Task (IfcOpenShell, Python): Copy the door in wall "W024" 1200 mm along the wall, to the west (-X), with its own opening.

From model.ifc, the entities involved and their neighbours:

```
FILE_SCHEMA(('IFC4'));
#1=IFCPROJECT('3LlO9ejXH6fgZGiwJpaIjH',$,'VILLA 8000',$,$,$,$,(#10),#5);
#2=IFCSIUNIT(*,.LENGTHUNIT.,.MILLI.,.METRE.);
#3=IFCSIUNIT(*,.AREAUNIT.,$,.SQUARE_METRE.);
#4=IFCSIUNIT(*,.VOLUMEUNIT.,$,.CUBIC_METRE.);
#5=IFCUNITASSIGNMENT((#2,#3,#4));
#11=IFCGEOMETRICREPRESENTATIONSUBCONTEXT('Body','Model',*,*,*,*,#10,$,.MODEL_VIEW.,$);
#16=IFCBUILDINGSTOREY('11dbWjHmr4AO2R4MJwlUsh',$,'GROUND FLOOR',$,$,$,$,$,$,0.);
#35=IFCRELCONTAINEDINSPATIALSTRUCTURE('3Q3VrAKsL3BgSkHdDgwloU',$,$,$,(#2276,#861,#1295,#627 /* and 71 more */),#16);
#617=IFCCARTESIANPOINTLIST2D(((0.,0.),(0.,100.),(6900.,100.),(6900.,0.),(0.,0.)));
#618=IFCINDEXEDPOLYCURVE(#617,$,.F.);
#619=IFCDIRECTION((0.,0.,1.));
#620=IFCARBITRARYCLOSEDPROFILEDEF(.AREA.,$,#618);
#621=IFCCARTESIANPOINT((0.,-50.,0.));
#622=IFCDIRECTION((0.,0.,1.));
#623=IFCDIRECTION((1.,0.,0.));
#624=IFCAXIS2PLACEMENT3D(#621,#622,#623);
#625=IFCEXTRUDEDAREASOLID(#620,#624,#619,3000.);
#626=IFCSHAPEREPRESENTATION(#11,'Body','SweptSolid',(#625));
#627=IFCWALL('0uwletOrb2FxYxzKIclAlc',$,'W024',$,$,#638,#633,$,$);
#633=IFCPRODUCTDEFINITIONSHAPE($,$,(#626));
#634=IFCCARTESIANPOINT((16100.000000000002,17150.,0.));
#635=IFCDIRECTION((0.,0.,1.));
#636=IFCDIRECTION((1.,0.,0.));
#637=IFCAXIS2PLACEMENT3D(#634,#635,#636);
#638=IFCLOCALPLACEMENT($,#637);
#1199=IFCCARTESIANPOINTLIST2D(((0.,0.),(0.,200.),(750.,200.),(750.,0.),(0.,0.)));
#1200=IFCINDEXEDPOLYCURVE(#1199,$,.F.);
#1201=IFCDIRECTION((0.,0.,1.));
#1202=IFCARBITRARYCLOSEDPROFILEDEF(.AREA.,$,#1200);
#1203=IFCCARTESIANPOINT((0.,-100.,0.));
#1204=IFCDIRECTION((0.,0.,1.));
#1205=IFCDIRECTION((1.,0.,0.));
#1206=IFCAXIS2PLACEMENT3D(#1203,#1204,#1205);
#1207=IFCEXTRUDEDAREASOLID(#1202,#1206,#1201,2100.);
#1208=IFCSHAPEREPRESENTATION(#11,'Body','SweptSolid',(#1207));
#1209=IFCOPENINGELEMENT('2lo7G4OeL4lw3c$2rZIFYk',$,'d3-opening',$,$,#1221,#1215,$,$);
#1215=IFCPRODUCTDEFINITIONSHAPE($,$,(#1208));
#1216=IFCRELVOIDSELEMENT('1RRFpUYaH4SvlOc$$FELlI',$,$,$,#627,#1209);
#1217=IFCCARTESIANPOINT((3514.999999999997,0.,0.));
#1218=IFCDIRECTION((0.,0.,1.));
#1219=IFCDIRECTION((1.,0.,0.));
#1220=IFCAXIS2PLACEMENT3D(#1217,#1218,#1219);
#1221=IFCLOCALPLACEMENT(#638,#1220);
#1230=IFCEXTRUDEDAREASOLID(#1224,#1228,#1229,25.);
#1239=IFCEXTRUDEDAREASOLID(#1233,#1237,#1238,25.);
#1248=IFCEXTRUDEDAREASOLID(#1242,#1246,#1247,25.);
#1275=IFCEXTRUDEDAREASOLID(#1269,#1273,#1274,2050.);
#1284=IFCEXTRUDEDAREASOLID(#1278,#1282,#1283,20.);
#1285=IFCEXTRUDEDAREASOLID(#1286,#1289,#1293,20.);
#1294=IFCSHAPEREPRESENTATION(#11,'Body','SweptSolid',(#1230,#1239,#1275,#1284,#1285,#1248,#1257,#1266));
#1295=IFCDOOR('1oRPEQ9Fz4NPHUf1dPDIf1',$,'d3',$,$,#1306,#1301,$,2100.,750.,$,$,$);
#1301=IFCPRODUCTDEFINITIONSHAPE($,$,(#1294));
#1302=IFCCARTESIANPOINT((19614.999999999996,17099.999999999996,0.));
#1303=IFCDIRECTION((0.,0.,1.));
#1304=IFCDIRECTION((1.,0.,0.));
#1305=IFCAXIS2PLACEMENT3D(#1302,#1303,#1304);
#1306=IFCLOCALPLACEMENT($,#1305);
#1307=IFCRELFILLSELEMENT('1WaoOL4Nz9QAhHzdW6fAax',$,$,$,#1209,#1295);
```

```python
import ifcopenshell
import ifcopenshell.api.feature
import ifcopenshell.api.geometry
import ifcopenshell.api.root
import ifcopenshell.geom
import ifcopenshell.util.element
import ifcopenshell.util.placement
import ifcopenshell.util.shape

model = ifcopenshell.open("model.ifc")
settings = ifcopenshell.geom.settings()


def volume(element):
    """Net volume in cubic metres, openings subtracted."""
    shape = ifcopenshell.geom.create_shape(settings, element)
    return ifcopenshell.util.shape.get_volume(shape.geometry)


door = model.by_guid("1oRPEQ9Fz4NPHUf1dPDIf1")
opening = door.FillsVoids[0].RelatingOpeningElement
wall = opening.VoidsElements[0].RelatingBuildingElement
before = volume(wall)
shift = ifcopenshell.util.placement.get_local_placement(wall.ObjectPlacement)[:3, 0] * -1200.0

# copy_class copies the void relationship, type, container and properties, but no geometry.
new_opening = ifcopenshell.api.root.copy_class(model, product=opening)
new_opening.Representation = ifcopenshell.util.element.copy_deep(
    model, opening.Representation, exclude=["IfcGeometricRepresentationContext", "IfcRepresentationMap"]
)
new_door = ifcopenshell.api.root.copy_class(model, product=door)
new_door.Representation = ifcopenshell.util.element.copy_deep(
    model, door.Representation, exclude=["IfcGeometricRepresentationContext", "IfcRepresentationMap"]
)
ifcopenshell.api.feature.add_filling(model, opening=new_opening, element=new_door)

for old, new in ((opening, new_opening), (door, new_door)):
    matrix = ifcopenshell.util.placement.get_local_placement(old.ObjectPlacement)
    matrix[:3, 3] += shift
    ifcopenshell.api.geometry.edit_object_placement(model, product=new, matrix=matrix, is_si=False)

after = volume(wall)

print(f"wall volume {before:.3f} -> {after:.3f} m3")

model.write("model_v2.ifc")
```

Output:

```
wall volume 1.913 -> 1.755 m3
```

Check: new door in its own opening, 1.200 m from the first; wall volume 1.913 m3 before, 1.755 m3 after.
